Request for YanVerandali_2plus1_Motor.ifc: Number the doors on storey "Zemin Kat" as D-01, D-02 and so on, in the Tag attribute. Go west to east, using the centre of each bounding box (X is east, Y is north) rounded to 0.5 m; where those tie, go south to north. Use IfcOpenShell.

First a look at what the model holds.

```python
import ifcopenshell
import ifcopenshell.util.element
import ifcopenshell.util.placement

model = ifcopenshell.open("YanVerandali_2plus1_Motor.ifc")
print(model.schema)
storey = next(s for s in model.by_type("IfcBuildingStorey") if s.Name == "Zemin Kat")
doors = [e for e in ifcopenshell.util.element.get_decomposition(storey) if e.is_a("IfcDoor")]
for e in sorted(doors, key=lambda e: e.id()):
    origin = ifcopenshell.util.placement.get_local_placement(e.ObjectPlacement)[:3, 3]
    print(e.id(), e.Tag, e.Name, origin.round(2) + 0.0, sep=" | ")
```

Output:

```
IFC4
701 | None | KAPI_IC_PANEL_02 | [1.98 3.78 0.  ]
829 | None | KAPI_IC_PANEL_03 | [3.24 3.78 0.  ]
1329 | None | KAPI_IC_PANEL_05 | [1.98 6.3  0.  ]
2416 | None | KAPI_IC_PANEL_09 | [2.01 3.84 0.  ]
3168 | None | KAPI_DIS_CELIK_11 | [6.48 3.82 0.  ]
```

```python
import ifcopenshell
import ifcopenshell.geom
import ifcopenshell.util.element
import ifcopenshell.util.shape

model = ifcopenshell.open("YanVerandali_2plus1_Motor.ifc")
settings = ifcopenshell.geom.settings()
settings.set("use-world-coords", True)


def centre(element):
    shape = ifcopenshell.geom.create_shape(settings, element)
    return ifcopenshell.util.shape.get_bbox_centroid(shape.geometry)


storey = next(s for s in model.by_type("IfcBuildingStorey") if s.Name == "Zemin Kat")
doors = [e for e in ifcopenshell.util.element.get_decomposition(storey) if e.is_a("IfcDoor")]

# Insertion points can sit at a corner or the storey origin, so sort by the geometry (in metres).
centres = {e: centre(e) for e in doors}
doors.sort(key=lambda e: (round(centres[e][0] / 0.5), centres[e][1]))

for i, e in enumerate(doors, start=1):
    number = f"D-{i:02d}"
    e.Tag = number
    print(e.id(), number)

model.write("YanVerandali_2plus1_Motor_rev.ifc")
```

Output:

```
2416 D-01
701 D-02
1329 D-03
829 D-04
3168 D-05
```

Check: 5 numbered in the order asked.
